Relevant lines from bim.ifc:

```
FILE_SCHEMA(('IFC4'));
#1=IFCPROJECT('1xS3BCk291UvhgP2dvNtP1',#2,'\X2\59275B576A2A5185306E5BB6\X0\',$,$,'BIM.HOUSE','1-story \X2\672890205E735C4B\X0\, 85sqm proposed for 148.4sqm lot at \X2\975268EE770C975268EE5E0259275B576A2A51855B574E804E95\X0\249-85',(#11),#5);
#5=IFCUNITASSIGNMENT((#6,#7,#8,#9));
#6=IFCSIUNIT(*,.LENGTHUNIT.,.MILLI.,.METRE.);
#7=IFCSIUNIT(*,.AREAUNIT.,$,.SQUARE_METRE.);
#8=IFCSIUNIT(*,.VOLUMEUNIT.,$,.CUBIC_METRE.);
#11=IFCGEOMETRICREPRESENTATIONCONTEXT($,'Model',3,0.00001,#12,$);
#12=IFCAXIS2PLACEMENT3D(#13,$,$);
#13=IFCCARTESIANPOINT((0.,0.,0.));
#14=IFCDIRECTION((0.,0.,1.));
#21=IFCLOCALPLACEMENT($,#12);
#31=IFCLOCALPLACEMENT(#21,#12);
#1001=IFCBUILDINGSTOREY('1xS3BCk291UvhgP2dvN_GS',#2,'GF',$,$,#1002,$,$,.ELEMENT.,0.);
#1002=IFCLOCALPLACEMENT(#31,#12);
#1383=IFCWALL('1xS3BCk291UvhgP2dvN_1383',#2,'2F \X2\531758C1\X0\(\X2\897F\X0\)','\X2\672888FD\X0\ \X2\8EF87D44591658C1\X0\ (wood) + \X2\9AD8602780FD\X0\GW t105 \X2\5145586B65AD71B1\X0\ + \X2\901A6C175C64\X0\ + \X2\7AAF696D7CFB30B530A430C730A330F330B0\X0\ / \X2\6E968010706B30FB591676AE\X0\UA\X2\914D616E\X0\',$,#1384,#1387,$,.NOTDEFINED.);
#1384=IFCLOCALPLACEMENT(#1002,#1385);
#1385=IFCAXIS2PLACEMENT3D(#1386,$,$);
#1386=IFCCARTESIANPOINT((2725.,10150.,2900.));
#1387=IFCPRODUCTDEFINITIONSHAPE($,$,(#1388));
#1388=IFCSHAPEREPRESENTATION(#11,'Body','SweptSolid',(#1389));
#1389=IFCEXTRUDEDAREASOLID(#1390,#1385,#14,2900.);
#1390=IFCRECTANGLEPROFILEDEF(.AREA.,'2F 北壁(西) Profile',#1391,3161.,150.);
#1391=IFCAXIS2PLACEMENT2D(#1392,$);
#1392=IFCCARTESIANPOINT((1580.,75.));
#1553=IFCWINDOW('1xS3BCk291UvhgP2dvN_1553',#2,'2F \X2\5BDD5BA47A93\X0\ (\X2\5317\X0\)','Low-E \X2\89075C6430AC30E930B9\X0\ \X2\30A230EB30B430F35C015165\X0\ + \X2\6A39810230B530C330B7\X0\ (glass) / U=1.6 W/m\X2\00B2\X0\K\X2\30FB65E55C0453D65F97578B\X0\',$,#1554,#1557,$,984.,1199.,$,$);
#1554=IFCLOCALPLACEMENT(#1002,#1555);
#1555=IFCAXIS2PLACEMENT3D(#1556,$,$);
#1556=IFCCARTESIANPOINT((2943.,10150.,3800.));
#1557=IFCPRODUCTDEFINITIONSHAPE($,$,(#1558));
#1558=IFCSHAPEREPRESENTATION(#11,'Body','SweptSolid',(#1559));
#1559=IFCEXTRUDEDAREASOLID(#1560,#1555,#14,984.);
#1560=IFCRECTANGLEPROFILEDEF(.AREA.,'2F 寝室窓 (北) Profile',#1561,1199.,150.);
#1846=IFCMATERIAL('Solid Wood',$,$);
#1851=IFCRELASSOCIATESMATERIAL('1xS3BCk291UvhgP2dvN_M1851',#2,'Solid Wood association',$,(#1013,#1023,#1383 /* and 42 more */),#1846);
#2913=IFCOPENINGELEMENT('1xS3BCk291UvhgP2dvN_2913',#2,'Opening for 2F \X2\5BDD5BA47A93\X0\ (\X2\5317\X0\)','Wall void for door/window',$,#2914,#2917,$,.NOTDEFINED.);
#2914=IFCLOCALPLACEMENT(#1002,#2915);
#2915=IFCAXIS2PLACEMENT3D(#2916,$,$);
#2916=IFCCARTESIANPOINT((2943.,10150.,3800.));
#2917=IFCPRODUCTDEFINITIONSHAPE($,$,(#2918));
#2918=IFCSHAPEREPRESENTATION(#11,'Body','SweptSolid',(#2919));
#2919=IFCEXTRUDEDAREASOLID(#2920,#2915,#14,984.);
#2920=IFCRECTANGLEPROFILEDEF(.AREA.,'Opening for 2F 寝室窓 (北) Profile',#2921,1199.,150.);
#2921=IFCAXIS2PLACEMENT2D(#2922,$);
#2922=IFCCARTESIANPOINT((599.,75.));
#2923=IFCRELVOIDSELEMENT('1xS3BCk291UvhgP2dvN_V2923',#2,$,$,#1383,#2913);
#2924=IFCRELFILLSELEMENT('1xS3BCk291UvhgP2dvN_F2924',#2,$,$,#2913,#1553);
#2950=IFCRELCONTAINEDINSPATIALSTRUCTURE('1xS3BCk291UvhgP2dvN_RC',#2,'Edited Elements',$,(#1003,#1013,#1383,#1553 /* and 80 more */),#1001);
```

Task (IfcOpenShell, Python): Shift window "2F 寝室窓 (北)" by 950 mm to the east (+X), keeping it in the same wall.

```python
import ifcopenshell
import ifcopenshell.api.geometry
import ifcopenshell.util.placement
import ifcopenshell.util.unit

model = ifcopenshell.open("bim.ifc")
unit_scale = ifcopenshell.util.unit.calculate_unit_scale(model)

window = model.by_guid("1xS3BCk291UvhgP2dvN_1553")
opening = window.FillsVoids[0].RelatingOpeningElement
wall = opening.VoidsElements[0].RelatingBuildingElement

wall_matrix = ifcopenshell.util.placement.get_local_placement(wall.ObjectPlacement)
shift = wall_matrix[:3, 0] * 0.95 / unit_scale
before = ifcopenshell.util.placement.get_local_placement(window.ObjectPlacement)[:3, 3].copy()

# The window is not placed relative to its opening, so move both.
for product in (opening, window):
    matrix = ifcopenshell.util.placement.get_local_placement(product.ObjectPlacement)
    matrix[:3, 3] += shift
    ifcopenshell.api.geometry.edit_object_placement(model, product=product, matrix=matrix, is_si=False)

after = ifcopenshell.util.placement.get_local_placement(window.ObjectPlacement)[:3, 3]
print("window moved by", (after - before).round(3) + 0.0)

model.write("bim_v2.ifc")
```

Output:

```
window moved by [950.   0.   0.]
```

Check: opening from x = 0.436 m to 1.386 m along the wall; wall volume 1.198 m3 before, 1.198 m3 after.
